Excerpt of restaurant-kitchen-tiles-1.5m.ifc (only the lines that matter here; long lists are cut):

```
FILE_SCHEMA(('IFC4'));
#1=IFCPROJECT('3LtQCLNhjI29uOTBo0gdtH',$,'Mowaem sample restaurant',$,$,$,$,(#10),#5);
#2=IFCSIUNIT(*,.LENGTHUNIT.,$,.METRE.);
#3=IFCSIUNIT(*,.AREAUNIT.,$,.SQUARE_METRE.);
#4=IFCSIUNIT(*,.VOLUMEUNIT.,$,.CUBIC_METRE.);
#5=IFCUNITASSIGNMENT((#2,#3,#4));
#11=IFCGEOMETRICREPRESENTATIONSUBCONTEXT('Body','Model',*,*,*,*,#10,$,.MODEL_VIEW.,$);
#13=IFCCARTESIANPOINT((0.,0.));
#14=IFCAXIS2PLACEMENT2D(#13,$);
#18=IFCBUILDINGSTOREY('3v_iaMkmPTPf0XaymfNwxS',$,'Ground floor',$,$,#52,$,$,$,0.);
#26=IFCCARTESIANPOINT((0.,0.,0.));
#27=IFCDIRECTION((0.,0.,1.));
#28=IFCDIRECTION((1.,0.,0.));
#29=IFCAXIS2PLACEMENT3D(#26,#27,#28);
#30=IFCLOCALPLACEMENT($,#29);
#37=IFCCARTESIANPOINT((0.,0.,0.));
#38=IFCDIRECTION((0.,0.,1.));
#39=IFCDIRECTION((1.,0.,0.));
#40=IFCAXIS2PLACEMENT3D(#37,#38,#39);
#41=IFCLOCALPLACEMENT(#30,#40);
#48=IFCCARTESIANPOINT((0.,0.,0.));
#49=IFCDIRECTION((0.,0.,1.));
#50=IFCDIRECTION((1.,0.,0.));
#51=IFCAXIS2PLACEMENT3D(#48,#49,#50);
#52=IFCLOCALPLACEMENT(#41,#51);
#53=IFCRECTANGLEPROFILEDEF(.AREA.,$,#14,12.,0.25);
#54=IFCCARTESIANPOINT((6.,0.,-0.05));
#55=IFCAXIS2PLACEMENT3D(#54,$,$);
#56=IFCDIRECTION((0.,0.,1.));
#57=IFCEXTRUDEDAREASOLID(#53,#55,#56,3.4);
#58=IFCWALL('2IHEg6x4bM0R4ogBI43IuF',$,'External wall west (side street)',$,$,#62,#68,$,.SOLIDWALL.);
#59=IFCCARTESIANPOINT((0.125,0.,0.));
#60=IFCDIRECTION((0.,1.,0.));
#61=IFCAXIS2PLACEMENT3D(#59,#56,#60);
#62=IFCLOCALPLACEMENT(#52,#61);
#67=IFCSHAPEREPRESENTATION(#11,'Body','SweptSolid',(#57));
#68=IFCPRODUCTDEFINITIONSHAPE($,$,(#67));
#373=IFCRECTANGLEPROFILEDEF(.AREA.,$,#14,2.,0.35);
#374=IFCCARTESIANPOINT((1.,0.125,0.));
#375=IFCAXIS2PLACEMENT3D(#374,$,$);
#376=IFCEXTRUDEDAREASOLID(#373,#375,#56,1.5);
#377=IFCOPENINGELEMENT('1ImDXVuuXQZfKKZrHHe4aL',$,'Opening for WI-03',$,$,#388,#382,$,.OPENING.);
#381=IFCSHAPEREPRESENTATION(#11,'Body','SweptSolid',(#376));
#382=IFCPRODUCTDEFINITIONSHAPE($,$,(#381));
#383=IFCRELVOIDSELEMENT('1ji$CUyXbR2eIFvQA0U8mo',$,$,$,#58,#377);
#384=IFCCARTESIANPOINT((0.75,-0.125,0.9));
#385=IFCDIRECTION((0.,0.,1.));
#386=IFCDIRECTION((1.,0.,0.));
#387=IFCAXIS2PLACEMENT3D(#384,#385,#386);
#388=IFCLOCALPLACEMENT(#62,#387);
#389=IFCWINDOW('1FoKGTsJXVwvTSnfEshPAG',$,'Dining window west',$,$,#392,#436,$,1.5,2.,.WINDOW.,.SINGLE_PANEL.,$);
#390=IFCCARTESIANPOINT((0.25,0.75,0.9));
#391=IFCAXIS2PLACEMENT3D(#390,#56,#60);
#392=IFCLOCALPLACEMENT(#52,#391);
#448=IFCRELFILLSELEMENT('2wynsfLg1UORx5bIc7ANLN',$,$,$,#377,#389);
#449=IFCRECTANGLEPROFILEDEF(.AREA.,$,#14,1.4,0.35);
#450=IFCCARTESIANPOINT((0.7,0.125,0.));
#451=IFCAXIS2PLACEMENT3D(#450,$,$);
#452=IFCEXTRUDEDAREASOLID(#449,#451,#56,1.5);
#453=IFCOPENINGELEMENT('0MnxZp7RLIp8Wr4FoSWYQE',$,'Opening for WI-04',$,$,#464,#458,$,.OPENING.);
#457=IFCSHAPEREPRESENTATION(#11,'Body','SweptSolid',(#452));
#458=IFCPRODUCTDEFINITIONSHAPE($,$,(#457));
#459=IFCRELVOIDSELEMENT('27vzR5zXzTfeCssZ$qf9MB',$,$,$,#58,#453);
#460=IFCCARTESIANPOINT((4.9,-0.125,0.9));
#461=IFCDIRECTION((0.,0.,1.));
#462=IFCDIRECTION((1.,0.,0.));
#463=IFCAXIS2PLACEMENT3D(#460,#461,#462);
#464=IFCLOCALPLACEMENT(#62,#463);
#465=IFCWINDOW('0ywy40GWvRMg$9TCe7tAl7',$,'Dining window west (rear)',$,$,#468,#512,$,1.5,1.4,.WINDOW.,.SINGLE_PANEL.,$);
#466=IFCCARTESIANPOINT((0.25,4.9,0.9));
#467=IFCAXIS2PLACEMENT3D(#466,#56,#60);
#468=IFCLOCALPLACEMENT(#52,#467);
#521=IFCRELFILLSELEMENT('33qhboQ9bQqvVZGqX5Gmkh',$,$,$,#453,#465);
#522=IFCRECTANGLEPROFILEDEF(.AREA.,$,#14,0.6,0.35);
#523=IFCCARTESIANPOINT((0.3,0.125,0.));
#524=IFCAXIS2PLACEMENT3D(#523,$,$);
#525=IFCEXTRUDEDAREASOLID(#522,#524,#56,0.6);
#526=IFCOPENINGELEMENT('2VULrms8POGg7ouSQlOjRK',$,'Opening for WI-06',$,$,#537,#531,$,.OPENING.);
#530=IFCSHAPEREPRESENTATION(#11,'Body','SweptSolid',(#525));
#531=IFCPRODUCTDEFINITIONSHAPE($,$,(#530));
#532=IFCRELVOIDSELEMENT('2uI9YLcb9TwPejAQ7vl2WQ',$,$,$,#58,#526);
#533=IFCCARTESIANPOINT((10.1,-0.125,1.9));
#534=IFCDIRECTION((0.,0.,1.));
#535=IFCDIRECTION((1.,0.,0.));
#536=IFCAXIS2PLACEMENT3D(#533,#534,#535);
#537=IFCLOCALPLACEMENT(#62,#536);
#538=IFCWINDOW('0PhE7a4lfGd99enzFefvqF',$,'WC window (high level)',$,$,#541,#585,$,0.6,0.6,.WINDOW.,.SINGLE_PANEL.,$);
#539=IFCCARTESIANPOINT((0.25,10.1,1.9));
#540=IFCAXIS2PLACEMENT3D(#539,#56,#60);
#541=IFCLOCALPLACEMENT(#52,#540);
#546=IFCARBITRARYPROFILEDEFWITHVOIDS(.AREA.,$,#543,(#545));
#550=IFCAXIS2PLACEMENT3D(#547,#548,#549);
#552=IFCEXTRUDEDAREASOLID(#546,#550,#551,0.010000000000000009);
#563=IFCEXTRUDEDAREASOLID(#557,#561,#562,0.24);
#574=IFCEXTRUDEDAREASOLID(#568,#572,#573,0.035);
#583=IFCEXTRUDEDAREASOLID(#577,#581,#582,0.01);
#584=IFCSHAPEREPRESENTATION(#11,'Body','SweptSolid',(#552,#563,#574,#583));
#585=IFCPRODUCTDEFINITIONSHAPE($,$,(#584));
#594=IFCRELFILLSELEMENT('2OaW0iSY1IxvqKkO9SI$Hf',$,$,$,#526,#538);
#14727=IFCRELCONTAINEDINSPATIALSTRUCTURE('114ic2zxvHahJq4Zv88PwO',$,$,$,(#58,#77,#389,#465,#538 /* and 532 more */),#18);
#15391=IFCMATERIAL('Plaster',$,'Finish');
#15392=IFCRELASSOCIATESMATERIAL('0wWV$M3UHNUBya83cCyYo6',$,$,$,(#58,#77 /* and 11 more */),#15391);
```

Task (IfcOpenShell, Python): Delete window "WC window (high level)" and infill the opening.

```python
import ifcopenshell
import ifcopenshell.api.feature
import ifcopenshell.api.root
import ifcopenshell.geom
import ifcopenshell.util.shape

model = ifcopenshell.open("restaurant-kitchen-tiles-1.5m.ifc")
settings = ifcopenshell.geom.settings()


def volume(element):
    """Net volume in cubic metres, openings subtracted."""
    shape = ifcopenshell.geom.create_shape(settings, element)
    return ifcopenshell.util.shape.get_volume(shape.geometry)


window = model.by_guid("0PhE7a4lfGd99enzFefvqF")
opening = window.FillsVoids[0].RelatingOpeningElement
wall = opening.VoidsElements[0].RelatingBuildingElement
before = volume(wall)

ifcopenshell.api.root.remove_product(model, product=window)
ifcopenshell.api.feature.remove_feature(model, feature=opening)

after = volume(wall)

print(f"wall volume {before:.3f} -> {after:.3f} m3")

model.write("restaurant-kitchen-tiles-1.5m_rev.ifc")
```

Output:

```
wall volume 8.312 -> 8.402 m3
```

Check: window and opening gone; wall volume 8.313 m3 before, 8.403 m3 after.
